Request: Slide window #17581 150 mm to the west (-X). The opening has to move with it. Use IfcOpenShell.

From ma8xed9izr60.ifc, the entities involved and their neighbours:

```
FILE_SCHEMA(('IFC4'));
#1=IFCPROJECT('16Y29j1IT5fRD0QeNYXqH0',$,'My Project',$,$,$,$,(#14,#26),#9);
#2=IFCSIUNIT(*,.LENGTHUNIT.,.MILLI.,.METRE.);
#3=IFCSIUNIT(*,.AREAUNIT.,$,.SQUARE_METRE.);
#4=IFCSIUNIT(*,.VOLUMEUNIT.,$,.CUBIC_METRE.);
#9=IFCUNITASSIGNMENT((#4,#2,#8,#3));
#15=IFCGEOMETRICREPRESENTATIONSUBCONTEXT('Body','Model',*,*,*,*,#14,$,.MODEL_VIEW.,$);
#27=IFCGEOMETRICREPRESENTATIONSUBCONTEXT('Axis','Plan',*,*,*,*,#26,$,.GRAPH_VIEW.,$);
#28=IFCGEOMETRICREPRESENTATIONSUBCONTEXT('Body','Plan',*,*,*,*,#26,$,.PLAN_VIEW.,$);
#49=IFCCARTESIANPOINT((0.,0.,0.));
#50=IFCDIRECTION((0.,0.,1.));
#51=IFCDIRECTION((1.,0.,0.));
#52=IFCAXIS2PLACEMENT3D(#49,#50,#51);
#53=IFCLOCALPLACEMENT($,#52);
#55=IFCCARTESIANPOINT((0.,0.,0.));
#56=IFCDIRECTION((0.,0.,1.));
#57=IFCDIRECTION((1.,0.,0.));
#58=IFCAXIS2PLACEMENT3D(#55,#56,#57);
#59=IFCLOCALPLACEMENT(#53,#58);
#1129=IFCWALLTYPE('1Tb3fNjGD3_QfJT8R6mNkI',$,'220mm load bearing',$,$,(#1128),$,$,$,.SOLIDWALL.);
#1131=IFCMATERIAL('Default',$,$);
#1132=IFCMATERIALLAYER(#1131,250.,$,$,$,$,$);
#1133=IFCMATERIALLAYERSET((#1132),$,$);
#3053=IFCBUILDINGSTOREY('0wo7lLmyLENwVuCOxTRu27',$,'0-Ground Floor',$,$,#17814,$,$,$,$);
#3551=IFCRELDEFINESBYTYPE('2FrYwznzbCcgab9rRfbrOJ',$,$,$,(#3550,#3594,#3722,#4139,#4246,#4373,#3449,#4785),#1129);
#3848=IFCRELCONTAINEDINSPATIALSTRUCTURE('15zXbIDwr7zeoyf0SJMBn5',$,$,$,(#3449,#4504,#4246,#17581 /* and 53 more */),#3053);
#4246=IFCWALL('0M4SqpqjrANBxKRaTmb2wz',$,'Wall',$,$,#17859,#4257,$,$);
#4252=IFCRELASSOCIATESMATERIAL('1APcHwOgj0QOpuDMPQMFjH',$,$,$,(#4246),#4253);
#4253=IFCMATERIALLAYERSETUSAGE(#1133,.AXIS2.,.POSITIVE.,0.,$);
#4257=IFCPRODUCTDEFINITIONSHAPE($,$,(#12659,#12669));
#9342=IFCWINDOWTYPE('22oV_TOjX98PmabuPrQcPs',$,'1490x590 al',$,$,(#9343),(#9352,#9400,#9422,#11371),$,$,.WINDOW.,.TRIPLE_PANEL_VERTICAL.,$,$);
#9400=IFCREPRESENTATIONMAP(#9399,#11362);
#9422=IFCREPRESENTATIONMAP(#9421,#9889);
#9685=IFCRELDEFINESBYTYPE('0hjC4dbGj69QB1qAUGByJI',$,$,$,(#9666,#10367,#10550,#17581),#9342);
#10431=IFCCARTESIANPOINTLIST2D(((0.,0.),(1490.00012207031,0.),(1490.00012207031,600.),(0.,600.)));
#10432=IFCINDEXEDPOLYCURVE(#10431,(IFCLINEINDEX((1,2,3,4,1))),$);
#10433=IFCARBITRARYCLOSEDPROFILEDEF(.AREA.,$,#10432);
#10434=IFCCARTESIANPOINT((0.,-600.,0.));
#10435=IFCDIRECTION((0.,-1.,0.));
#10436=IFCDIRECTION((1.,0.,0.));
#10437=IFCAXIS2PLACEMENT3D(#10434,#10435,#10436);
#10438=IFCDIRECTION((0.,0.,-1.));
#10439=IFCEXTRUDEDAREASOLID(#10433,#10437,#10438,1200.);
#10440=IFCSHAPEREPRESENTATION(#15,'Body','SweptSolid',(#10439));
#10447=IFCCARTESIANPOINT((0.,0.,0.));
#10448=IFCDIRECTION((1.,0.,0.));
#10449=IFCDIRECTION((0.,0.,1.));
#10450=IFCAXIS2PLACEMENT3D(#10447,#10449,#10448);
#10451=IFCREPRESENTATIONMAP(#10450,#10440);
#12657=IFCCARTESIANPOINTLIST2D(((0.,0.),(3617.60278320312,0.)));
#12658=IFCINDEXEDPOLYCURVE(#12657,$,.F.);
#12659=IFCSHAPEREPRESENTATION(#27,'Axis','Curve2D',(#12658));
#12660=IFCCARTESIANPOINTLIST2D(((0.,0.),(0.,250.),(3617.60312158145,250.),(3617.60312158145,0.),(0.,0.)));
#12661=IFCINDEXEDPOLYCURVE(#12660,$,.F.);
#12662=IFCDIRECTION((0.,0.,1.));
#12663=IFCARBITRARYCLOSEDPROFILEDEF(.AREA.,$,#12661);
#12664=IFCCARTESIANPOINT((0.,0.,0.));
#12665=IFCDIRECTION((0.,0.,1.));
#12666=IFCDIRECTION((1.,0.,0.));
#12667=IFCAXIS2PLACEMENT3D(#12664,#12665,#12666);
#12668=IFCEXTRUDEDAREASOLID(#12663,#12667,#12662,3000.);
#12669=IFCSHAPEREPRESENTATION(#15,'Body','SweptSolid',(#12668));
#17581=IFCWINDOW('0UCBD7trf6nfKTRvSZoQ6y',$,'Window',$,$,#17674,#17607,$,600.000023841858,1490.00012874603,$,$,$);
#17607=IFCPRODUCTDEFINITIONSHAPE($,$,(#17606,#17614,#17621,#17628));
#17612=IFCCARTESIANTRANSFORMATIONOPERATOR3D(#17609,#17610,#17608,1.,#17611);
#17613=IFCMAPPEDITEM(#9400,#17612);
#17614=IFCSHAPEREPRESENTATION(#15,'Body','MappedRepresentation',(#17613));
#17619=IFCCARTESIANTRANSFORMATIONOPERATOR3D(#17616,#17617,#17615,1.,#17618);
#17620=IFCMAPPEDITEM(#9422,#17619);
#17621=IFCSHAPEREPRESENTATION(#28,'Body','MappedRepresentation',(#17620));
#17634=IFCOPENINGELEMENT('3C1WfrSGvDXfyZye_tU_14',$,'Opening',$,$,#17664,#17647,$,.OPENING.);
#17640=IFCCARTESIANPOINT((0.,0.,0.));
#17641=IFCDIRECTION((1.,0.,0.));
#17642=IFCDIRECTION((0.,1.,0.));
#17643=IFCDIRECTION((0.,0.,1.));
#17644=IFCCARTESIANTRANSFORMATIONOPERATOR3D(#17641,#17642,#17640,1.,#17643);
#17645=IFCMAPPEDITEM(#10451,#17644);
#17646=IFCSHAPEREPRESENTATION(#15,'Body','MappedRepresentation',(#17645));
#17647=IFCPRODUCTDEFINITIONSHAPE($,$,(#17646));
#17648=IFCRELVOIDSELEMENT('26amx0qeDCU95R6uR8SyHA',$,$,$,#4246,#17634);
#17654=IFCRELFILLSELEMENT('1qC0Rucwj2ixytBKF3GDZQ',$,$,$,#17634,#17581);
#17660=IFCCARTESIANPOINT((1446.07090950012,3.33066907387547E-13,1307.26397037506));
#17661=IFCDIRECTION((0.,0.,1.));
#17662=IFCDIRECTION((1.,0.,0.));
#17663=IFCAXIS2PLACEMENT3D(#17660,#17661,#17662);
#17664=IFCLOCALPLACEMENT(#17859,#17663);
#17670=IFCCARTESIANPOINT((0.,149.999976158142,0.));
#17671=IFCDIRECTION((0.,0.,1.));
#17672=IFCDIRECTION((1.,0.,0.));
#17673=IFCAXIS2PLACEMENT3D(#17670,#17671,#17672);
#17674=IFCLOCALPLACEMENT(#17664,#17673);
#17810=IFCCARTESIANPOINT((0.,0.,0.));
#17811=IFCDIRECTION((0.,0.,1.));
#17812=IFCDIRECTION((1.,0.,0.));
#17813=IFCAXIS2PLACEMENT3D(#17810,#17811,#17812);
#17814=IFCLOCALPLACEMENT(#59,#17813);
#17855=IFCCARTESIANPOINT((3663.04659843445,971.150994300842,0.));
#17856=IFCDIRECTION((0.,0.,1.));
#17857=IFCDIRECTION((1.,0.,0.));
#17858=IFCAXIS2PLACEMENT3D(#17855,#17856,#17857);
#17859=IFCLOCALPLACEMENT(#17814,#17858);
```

```python
import ifcopenshell
import ifcopenshell.api.geometry
import ifcopenshell.util.placement
import ifcopenshell.util.unit

model = ifcopenshell.open("ma8xed9izr60.ifc")
unit_scale = ifcopenshell.util.unit.calculate_unit_scale(model)

window = model.by_guid("0UCBD7trf6nfKTRvSZoQ6y")
opening = window.FillsVoids[0].RelatingOpeningElement
wall = opening.VoidsElements[0].RelatingBuildingElement

wall_matrix = ifcopenshell.util.placement.get_local_placement(wall.ObjectPlacement)
shift = wall_matrix[:3, 0] * -0.15 / unit_scale
before = ifcopenshell.util.placement.get_local_placement(window.ObjectPlacement)[:3, 3].copy()

# The window is placed relative to its opening, so it follows when the opening moves.
matrix = ifcopenshell.util.placement.get_local_placement(opening.ObjectPlacement)
matrix[:3, 3] += shift
ifcopenshell.api.geometry.edit_object_placement(
    model, product=opening, matrix=matrix, is_si=False, should_transform_children=True
)

after = ifcopenshell.util.placement.get_local_placement(window.ObjectPlacement)[:3, 3]
print("window moved by", (after - before).round(3) + 0.0)

model.write("ma8xed9izr60_edited.ifc")
```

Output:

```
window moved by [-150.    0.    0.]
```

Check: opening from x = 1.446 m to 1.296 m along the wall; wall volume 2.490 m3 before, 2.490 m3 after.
